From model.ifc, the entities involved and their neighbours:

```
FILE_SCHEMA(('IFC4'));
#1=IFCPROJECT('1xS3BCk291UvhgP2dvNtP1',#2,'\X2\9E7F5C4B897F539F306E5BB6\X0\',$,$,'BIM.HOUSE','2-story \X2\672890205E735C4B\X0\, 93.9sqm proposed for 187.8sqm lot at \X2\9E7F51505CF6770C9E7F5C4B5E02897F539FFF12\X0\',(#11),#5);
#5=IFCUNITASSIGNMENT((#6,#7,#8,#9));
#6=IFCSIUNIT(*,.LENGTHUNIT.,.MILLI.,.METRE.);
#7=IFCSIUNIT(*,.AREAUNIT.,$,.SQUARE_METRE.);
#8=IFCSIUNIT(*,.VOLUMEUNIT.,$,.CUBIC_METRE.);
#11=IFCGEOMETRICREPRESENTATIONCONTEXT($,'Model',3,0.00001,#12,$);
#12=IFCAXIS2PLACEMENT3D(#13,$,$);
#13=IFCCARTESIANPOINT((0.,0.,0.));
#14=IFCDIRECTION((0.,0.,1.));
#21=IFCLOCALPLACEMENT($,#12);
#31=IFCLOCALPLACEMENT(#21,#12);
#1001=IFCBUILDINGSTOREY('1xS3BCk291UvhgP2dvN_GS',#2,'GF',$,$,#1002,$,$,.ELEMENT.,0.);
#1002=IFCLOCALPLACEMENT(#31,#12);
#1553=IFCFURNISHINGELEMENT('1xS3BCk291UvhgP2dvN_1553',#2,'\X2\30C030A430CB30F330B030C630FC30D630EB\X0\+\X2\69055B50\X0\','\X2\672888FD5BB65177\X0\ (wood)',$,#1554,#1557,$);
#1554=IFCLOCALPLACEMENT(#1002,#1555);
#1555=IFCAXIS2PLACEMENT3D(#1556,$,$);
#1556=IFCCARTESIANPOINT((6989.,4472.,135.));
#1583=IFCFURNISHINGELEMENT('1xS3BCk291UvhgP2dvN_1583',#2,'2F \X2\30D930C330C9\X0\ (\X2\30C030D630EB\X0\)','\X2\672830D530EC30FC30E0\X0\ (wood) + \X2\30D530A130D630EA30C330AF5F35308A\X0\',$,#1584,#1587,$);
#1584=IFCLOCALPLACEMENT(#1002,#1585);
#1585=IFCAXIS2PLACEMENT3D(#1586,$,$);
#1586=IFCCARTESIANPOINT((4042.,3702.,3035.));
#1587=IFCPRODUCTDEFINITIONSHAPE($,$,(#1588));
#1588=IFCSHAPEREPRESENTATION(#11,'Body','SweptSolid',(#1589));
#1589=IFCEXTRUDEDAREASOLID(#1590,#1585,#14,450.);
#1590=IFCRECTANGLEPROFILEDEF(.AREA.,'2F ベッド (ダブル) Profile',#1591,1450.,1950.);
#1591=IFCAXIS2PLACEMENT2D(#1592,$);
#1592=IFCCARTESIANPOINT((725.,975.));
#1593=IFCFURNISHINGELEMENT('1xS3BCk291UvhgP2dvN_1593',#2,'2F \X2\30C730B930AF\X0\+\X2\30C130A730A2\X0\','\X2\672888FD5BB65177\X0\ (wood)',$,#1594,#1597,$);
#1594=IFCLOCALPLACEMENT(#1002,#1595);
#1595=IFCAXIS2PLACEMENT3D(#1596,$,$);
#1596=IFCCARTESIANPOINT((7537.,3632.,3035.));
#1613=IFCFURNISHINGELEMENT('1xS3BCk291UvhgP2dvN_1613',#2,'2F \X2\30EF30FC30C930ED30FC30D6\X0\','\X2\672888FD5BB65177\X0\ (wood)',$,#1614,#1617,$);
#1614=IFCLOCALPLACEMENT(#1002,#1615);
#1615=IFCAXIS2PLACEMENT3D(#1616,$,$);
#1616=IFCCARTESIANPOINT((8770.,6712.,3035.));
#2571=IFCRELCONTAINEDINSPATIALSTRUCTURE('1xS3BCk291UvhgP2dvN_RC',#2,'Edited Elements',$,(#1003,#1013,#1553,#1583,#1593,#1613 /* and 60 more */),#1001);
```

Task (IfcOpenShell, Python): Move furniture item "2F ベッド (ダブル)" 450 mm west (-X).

```python
import ifcopenshell
import ifcopenshell.api.geometry
import ifcopenshell.util.placement
import ifcopenshell.util.unit

model = ifcopenshell.open("model.ifc")
unit_scale = ifcopenshell.util.unit.calculate_unit_scale(model)

item = model.by_guid("1xS3BCk291UvhgP2dvN_1583")
matrix = ifcopenshell.util.placement.get_local_placement(item.ObjectPlacement)
matrix[0, 3] -= 0.45 / unit_scale
ifcopenshell.api.geometry.edit_object_placement(model, product=item, matrix=matrix, is_si=False)

print(ifcopenshell.util.placement.get_local_placement(item.ObjectPlacement).round(3) + 0.0)

model.write("model_v2.ifc")
```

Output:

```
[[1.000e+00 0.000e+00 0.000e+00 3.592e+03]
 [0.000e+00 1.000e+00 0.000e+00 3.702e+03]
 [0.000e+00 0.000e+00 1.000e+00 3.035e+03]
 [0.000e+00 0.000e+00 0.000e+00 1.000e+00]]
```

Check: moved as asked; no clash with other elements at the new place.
